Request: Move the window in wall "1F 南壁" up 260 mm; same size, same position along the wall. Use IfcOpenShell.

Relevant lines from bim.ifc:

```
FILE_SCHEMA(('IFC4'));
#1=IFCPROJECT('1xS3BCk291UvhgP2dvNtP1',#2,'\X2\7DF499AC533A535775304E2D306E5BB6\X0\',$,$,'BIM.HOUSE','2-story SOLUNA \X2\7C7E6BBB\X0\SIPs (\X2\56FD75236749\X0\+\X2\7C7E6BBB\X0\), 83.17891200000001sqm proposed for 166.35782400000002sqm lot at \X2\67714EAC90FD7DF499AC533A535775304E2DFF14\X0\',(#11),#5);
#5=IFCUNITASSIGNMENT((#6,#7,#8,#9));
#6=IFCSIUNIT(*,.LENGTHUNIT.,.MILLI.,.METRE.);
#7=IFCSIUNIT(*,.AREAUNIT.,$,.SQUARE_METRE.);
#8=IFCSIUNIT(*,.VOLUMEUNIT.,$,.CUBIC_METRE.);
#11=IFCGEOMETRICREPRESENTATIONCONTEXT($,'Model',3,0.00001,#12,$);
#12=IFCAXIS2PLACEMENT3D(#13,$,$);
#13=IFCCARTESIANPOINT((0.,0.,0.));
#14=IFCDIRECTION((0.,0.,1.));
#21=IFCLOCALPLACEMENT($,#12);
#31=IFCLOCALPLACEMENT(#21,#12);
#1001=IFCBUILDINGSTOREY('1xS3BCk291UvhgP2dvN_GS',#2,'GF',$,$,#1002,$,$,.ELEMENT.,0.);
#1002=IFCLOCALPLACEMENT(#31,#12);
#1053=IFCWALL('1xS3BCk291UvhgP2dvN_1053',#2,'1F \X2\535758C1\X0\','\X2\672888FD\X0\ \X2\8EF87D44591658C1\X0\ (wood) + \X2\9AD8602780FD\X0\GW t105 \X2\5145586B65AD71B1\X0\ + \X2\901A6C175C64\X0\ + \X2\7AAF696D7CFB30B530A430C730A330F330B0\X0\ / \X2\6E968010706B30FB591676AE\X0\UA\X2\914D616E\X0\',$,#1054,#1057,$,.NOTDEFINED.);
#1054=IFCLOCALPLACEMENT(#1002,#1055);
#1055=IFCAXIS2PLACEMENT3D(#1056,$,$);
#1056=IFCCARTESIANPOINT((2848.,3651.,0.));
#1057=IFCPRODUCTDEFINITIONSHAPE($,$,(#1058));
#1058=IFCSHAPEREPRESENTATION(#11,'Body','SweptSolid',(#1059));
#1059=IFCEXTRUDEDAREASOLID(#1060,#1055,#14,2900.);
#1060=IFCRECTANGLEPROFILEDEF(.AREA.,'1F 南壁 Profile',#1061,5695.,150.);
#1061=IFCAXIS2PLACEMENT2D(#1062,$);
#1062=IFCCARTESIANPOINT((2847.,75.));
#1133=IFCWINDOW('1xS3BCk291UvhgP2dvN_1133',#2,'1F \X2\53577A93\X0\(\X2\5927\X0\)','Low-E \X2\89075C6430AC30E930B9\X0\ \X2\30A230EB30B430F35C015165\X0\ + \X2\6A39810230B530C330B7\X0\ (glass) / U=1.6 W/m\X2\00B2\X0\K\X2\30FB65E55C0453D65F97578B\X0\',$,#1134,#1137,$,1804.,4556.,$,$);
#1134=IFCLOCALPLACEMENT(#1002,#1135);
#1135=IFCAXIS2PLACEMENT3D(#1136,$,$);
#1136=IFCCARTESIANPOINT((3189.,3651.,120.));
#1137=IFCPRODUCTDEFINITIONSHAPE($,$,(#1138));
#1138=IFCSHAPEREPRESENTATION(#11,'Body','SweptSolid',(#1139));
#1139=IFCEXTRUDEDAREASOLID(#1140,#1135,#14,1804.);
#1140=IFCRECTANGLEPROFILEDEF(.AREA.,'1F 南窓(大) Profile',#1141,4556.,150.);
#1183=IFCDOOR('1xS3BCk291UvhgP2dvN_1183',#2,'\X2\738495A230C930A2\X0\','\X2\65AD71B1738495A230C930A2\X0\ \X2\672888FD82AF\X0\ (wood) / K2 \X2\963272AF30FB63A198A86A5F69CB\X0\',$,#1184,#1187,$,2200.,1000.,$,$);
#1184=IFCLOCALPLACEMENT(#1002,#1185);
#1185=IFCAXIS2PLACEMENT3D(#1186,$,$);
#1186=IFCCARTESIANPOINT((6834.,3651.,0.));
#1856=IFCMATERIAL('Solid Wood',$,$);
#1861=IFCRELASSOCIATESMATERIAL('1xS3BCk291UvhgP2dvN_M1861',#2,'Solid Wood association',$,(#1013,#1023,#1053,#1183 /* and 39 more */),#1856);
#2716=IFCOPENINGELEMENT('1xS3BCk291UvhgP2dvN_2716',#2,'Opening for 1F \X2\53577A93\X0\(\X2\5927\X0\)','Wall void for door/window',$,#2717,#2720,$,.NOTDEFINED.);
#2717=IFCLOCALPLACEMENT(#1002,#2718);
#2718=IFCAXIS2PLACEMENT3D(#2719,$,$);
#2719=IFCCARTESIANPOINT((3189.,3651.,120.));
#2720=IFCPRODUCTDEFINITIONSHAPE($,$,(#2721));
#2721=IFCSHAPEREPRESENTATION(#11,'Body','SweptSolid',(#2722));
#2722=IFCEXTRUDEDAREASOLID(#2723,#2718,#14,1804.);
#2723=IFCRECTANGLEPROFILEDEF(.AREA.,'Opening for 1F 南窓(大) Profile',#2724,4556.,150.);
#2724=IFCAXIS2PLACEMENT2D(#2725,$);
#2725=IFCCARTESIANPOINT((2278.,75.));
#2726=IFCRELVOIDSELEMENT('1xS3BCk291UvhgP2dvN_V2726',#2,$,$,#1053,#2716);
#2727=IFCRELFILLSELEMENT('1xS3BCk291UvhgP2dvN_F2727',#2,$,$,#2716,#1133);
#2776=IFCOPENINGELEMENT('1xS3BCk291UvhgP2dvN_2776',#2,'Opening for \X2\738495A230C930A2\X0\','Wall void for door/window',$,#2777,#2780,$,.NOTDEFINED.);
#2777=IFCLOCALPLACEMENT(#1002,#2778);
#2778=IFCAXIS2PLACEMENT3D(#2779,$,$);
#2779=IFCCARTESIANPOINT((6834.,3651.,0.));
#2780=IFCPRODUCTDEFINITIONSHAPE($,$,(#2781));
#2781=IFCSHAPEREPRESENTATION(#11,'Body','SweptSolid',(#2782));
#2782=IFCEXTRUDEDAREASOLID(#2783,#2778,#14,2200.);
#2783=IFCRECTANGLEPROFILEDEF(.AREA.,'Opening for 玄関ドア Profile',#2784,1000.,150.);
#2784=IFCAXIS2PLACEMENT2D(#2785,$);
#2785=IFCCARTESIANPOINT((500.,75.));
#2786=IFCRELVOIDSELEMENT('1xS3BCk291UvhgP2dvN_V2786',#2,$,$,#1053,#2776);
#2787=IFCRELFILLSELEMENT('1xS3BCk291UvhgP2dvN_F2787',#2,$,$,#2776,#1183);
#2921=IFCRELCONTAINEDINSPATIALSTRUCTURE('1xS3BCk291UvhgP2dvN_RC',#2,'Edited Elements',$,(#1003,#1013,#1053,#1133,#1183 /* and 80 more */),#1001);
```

```python
import numpy as np
import ifcopenshell
import ifcopenshell.api.geometry
import ifcopenshell.util.placement
import ifcopenshell.util.unit

model = ifcopenshell.open("bim.ifc")
unit_scale = ifcopenshell.util.unit.calculate_unit_scale(model)

window = model.by_id(1133)
opening = window.FillsVoids[0].RelatingOpeningElement
dz = 0.26 / unit_scale

shift = np.array([0.0, 0.0, dz])
# The window is not placed relative to its opening, so move both.
for product in (opening, window):
    matrix = ifcopenshell.util.placement.get_local_placement(product.ObjectPlacement)
    matrix[:3, 3] += shift
    ifcopenshell.api.geometry.edit_object_placement(model, product=product, matrix=matrix, is_si=False)

print(f"moved by {dz * unit_scale:+.3f} m")

model.write("bim_rev.ifc")
```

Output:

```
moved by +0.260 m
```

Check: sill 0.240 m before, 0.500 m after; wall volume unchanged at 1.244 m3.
